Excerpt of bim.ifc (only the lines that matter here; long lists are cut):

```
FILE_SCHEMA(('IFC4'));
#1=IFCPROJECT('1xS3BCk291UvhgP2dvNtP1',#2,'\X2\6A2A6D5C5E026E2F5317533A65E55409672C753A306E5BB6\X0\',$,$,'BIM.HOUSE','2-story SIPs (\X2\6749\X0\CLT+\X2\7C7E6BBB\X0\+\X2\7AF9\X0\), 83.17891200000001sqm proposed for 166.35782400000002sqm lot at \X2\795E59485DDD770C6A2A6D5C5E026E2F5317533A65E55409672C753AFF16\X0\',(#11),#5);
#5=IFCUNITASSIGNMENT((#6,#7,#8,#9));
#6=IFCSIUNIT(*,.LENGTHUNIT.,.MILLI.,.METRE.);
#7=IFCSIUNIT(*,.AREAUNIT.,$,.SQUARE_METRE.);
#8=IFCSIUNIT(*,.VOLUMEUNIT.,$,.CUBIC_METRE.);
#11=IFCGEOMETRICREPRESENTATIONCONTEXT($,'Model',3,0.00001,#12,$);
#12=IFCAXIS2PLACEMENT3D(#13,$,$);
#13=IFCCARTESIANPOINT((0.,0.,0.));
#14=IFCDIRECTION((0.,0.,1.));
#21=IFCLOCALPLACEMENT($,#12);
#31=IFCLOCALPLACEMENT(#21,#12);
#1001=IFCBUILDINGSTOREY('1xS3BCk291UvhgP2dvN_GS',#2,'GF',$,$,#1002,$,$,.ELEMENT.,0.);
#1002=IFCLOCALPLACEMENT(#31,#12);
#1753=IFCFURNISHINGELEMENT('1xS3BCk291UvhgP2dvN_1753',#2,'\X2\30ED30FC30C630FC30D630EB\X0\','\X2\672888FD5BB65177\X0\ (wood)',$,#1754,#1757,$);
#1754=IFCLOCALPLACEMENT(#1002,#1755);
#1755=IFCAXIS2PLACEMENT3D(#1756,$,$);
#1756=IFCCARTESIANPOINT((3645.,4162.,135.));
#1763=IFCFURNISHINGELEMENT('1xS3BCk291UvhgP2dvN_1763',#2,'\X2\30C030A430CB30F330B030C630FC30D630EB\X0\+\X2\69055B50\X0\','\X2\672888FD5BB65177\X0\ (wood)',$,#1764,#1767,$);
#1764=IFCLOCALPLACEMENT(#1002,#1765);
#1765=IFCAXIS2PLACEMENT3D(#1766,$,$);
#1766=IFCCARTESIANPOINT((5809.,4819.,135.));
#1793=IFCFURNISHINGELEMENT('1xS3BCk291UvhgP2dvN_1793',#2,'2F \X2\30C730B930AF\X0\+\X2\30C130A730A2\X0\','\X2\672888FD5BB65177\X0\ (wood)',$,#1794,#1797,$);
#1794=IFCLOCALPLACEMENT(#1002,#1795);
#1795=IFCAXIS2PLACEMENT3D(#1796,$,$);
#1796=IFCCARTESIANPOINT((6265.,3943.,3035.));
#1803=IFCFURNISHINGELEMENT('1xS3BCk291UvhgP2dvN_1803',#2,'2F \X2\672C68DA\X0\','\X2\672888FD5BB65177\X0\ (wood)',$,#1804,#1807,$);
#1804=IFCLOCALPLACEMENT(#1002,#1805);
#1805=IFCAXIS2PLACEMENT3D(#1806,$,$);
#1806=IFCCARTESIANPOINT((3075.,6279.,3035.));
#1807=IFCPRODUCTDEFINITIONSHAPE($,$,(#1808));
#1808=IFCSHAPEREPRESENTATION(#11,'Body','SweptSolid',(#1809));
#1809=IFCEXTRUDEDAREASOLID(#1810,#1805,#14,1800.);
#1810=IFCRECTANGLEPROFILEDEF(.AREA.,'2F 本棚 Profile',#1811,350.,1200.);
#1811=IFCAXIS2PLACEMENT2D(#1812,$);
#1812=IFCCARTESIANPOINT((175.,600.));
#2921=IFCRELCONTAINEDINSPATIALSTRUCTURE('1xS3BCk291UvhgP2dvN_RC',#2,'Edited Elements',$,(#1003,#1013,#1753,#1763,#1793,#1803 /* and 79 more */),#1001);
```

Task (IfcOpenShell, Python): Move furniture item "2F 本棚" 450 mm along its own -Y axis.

```python
import ifcopenshell
import ifcopenshell.api.geometry
import ifcopenshell.util.placement
import ifcopenshell.util.unit

model = ifcopenshell.open("bim.ifc")
unit_scale = ifcopenshell.util.unit.calculate_unit_scale(model)

item = model.by_guid("1xS3BCk291UvhgP2dvN_1803")
matrix = ifcopenshell.util.placement.get_local_placement(item.ObjectPlacement)
matrix[:3, 3] -= matrix[:3, 1] * 0.45 / unit_scale
ifcopenshell.api.geometry.edit_object_placement(model, product=item, matrix=matrix, is_si=False)

print(ifcopenshell.util.placement.get_local_placement(item.ObjectPlacement).round(3) + 0.0)

model.write("bim-out.ifc")
```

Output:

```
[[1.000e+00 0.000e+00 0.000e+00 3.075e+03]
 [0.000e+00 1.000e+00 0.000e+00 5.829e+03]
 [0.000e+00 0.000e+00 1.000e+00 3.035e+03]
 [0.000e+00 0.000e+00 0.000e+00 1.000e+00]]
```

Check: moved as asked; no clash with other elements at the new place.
